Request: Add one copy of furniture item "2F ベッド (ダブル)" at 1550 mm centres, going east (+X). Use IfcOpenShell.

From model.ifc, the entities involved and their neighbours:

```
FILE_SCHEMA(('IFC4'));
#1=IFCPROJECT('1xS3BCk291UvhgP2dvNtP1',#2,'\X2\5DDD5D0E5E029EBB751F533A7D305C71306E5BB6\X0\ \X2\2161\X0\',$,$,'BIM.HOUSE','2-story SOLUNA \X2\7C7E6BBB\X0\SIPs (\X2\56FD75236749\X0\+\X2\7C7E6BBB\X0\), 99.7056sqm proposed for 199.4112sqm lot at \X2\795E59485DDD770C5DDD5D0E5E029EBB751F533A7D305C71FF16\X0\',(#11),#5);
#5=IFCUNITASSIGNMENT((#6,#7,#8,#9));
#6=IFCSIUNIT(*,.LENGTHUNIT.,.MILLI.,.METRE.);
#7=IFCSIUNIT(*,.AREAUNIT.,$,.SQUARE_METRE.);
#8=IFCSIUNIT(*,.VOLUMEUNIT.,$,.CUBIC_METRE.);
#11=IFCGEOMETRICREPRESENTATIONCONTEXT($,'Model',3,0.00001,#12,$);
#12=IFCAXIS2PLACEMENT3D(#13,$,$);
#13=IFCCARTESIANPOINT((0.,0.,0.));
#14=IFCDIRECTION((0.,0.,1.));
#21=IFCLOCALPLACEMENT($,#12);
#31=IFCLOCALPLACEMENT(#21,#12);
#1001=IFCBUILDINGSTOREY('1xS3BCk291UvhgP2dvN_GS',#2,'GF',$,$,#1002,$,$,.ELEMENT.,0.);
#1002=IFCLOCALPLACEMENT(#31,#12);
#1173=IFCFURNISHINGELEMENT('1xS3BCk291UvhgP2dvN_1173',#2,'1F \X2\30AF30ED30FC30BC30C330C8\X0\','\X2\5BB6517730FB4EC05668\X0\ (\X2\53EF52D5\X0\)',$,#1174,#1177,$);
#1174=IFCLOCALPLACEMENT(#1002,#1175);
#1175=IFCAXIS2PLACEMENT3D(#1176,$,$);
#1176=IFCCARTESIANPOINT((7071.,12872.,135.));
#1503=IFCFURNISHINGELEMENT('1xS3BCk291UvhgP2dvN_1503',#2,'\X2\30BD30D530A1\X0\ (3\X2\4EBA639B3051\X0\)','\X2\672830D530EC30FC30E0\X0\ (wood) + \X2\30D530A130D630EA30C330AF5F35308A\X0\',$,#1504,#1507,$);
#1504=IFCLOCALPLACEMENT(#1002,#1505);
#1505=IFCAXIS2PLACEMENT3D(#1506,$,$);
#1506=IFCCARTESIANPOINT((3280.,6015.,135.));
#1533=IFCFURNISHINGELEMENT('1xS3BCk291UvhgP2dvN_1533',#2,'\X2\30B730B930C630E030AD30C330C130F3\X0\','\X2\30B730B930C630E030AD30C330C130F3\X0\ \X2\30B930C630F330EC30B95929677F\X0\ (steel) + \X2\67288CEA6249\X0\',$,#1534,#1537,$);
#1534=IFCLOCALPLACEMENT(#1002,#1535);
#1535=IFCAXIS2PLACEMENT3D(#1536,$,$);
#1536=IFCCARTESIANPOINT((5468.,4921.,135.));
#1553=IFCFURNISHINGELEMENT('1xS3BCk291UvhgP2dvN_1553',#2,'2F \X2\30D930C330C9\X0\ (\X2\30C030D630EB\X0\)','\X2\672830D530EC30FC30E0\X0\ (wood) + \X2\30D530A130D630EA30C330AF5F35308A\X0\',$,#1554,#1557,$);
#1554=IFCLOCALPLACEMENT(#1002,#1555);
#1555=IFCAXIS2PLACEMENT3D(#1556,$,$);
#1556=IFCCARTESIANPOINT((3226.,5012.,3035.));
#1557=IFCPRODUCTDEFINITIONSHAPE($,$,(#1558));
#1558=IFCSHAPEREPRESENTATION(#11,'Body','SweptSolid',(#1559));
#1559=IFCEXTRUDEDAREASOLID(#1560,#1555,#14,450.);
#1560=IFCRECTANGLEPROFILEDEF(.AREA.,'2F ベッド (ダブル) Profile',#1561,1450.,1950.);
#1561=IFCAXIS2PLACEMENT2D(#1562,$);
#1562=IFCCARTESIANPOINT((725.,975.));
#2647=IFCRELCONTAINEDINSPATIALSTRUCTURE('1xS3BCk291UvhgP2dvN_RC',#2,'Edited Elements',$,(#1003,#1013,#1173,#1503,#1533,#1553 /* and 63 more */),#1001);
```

```python
import numpy as np
import ifcopenshell
import ifcopenshell.api.geometry
import ifcopenshell.api.root
import ifcopenshell.util.element
import ifcopenshell.util.placement

model = ifcopenshell.open("model.ifc")


def reuse_history(source, copy):
    """copy_class also copies each property set's owner history, people and application; keep the originals."""
    for rel in copy.IsDefinedBy:
        if rel.is_a("IfcRelDefinesByProperties") and (history := rel.RelatingPropertyDefinition.OwnerHistory):
            rel.RelatingPropertyDefinition.OwnerHistory = source.OwnerHistory
            ifcopenshell.util.element.remove_deep2(model, history)


source = model.by_id(1553)
base = ifcopenshell.util.placement.get_local_placement(source.ObjectPlacement)
step = np.array([1.0, 0.0, 0.0]) * 1550.0

for i in range(1, 2):
    copy = ifcopenshell.api.root.copy_class(model, product=source)
    copy.Representation = ifcopenshell.util.element.copy_deep(
        model, source.Representation, exclude=["IfcGeometricRepresentationContext", "IfcRepresentationMap"]
    )
    reuse_history(source, copy)
    matrix = base.copy()
    matrix[:3, 3] += i * step
    print("added at", matrix[:3, 3].round(3) + 0.0)
    ifcopenshell.api.geometry.edit_object_placement(model, product=copy, matrix=matrix, is_si=False)

model.write("model-out.ifc")
```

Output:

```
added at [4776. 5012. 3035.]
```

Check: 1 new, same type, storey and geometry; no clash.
